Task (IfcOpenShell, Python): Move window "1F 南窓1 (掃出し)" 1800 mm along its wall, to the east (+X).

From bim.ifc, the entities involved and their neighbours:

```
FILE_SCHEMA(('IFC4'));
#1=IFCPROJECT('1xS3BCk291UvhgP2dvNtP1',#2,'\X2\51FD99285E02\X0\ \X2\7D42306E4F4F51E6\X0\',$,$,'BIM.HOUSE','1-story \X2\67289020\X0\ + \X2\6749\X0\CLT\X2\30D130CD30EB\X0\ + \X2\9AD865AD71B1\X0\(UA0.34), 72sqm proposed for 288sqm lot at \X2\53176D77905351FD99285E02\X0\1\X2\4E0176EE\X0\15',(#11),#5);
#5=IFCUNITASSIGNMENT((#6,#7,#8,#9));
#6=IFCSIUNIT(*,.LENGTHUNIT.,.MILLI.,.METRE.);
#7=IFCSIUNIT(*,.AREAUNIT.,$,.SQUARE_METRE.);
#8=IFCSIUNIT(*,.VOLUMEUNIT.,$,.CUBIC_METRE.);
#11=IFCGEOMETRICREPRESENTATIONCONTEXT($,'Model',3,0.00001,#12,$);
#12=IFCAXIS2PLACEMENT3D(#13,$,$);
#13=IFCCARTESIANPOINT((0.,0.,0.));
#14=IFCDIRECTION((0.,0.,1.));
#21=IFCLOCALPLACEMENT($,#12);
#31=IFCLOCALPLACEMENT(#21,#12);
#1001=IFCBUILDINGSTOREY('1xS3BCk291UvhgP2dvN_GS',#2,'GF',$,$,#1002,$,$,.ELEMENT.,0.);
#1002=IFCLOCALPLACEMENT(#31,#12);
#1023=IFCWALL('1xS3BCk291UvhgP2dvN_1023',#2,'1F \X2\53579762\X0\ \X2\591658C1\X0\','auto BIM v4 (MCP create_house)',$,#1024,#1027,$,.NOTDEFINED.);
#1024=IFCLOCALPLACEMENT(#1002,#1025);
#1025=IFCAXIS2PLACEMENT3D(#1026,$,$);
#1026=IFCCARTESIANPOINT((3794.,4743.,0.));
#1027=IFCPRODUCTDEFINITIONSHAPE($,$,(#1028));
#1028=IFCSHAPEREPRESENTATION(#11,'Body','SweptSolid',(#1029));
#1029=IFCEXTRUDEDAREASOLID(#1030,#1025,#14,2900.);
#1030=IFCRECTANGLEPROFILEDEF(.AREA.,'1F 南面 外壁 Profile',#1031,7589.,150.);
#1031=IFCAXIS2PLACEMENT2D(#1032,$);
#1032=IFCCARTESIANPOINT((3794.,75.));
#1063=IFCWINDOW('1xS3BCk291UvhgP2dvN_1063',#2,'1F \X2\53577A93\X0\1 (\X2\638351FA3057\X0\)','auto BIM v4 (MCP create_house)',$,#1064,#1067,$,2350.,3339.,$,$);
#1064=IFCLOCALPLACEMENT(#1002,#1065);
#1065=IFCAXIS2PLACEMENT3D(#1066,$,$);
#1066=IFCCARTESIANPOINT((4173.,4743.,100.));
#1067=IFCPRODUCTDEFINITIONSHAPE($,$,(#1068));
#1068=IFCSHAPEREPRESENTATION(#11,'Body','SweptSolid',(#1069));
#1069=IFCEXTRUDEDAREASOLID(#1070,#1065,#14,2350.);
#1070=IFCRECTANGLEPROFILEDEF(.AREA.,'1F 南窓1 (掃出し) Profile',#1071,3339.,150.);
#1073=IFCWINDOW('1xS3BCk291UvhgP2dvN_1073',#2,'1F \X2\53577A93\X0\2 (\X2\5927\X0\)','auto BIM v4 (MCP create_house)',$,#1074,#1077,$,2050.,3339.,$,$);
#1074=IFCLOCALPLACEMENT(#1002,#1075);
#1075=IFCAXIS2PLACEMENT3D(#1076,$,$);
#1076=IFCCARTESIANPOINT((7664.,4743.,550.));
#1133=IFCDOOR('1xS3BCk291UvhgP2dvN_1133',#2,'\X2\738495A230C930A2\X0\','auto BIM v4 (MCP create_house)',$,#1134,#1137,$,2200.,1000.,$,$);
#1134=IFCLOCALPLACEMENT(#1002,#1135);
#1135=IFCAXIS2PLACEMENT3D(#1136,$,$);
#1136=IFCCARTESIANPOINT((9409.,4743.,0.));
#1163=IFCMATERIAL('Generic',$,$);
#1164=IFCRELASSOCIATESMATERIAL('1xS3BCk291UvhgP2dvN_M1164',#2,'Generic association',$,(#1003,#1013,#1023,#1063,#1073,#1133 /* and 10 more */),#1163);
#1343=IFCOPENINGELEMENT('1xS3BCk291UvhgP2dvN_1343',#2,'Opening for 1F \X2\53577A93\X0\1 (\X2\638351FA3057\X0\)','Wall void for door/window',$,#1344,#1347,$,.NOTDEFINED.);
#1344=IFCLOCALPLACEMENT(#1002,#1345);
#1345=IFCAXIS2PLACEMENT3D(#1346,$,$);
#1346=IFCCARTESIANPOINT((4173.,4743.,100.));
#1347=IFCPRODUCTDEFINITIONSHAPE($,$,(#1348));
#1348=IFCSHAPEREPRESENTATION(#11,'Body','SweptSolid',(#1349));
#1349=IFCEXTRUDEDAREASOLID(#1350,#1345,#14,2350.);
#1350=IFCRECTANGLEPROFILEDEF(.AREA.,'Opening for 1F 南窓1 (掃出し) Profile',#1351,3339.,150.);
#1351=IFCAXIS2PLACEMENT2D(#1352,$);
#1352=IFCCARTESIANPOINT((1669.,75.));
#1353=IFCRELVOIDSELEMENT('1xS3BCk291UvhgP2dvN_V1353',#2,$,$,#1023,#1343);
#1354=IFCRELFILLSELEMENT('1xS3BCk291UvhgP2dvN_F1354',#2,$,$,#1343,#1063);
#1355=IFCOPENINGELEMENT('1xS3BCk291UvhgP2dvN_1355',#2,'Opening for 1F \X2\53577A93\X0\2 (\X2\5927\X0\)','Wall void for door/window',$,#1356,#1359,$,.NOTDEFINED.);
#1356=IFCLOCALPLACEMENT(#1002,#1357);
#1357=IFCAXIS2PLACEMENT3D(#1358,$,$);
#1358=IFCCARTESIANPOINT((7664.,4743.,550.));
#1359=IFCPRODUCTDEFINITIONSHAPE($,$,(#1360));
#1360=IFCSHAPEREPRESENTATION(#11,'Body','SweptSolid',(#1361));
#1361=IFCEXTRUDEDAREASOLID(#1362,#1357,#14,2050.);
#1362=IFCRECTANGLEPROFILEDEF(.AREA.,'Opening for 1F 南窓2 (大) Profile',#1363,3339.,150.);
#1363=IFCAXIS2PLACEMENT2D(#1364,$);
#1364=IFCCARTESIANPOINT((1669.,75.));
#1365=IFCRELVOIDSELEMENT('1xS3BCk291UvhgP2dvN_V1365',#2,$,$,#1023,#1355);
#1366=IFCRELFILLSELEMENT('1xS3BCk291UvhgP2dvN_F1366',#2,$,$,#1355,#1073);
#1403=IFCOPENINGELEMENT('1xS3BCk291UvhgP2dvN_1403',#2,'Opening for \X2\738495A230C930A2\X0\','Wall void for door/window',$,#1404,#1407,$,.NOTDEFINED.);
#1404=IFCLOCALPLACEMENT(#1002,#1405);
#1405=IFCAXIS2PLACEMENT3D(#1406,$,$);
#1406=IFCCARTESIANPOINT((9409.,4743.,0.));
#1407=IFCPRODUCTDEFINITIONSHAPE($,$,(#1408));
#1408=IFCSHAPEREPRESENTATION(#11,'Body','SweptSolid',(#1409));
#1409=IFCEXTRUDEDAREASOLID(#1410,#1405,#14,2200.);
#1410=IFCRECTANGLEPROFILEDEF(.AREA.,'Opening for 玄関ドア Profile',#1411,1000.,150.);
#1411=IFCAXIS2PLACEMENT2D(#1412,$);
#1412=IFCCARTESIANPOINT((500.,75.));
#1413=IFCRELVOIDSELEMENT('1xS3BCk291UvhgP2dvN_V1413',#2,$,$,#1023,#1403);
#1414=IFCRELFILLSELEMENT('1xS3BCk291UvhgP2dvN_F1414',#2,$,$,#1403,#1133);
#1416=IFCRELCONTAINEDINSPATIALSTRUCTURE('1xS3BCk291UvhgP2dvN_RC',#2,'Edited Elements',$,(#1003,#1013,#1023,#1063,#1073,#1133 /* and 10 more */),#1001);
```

```python
import ifcopenshell
import ifcopenshell.api.geometry
import ifcopenshell.util.placement

model = ifcopenshell.open("bim.ifc")

window = model.by_guid("1xS3BCk291UvhgP2dvN_1063")
opening = window.FillsVoids[0].RelatingOpeningElement
wall = opening.VoidsElements[0].RelatingBuildingElement

wall_matrix = ifcopenshell.util.placement.get_local_placement(wall.ObjectPlacement)
shift = wall_matrix[:3, 0] * 1800.0
before = ifcopenshell.util.placement.get_local_placement(window.ObjectPlacement)[:3, 3].copy()

# The window is not placed relative to its opening, so move both.
for product in (opening, window):
    matrix = ifcopenshell.util.placement.get_local_placement(product.ObjectPlacement)
    matrix[:3, 3] += shift
    ifcopenshell.api.geometry.edit_object_placement(model, product=product, matrix=matrix, is_si=False)

after = ifcopenshell.util.placement.get_local_placement(window.ObjectPlacement)[:3, 3]
print("window moved by", (after - before).round(3) + 0.0)

model.write("bim_edited.ifc")
```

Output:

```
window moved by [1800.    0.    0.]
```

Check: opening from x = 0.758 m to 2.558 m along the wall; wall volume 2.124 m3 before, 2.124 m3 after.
